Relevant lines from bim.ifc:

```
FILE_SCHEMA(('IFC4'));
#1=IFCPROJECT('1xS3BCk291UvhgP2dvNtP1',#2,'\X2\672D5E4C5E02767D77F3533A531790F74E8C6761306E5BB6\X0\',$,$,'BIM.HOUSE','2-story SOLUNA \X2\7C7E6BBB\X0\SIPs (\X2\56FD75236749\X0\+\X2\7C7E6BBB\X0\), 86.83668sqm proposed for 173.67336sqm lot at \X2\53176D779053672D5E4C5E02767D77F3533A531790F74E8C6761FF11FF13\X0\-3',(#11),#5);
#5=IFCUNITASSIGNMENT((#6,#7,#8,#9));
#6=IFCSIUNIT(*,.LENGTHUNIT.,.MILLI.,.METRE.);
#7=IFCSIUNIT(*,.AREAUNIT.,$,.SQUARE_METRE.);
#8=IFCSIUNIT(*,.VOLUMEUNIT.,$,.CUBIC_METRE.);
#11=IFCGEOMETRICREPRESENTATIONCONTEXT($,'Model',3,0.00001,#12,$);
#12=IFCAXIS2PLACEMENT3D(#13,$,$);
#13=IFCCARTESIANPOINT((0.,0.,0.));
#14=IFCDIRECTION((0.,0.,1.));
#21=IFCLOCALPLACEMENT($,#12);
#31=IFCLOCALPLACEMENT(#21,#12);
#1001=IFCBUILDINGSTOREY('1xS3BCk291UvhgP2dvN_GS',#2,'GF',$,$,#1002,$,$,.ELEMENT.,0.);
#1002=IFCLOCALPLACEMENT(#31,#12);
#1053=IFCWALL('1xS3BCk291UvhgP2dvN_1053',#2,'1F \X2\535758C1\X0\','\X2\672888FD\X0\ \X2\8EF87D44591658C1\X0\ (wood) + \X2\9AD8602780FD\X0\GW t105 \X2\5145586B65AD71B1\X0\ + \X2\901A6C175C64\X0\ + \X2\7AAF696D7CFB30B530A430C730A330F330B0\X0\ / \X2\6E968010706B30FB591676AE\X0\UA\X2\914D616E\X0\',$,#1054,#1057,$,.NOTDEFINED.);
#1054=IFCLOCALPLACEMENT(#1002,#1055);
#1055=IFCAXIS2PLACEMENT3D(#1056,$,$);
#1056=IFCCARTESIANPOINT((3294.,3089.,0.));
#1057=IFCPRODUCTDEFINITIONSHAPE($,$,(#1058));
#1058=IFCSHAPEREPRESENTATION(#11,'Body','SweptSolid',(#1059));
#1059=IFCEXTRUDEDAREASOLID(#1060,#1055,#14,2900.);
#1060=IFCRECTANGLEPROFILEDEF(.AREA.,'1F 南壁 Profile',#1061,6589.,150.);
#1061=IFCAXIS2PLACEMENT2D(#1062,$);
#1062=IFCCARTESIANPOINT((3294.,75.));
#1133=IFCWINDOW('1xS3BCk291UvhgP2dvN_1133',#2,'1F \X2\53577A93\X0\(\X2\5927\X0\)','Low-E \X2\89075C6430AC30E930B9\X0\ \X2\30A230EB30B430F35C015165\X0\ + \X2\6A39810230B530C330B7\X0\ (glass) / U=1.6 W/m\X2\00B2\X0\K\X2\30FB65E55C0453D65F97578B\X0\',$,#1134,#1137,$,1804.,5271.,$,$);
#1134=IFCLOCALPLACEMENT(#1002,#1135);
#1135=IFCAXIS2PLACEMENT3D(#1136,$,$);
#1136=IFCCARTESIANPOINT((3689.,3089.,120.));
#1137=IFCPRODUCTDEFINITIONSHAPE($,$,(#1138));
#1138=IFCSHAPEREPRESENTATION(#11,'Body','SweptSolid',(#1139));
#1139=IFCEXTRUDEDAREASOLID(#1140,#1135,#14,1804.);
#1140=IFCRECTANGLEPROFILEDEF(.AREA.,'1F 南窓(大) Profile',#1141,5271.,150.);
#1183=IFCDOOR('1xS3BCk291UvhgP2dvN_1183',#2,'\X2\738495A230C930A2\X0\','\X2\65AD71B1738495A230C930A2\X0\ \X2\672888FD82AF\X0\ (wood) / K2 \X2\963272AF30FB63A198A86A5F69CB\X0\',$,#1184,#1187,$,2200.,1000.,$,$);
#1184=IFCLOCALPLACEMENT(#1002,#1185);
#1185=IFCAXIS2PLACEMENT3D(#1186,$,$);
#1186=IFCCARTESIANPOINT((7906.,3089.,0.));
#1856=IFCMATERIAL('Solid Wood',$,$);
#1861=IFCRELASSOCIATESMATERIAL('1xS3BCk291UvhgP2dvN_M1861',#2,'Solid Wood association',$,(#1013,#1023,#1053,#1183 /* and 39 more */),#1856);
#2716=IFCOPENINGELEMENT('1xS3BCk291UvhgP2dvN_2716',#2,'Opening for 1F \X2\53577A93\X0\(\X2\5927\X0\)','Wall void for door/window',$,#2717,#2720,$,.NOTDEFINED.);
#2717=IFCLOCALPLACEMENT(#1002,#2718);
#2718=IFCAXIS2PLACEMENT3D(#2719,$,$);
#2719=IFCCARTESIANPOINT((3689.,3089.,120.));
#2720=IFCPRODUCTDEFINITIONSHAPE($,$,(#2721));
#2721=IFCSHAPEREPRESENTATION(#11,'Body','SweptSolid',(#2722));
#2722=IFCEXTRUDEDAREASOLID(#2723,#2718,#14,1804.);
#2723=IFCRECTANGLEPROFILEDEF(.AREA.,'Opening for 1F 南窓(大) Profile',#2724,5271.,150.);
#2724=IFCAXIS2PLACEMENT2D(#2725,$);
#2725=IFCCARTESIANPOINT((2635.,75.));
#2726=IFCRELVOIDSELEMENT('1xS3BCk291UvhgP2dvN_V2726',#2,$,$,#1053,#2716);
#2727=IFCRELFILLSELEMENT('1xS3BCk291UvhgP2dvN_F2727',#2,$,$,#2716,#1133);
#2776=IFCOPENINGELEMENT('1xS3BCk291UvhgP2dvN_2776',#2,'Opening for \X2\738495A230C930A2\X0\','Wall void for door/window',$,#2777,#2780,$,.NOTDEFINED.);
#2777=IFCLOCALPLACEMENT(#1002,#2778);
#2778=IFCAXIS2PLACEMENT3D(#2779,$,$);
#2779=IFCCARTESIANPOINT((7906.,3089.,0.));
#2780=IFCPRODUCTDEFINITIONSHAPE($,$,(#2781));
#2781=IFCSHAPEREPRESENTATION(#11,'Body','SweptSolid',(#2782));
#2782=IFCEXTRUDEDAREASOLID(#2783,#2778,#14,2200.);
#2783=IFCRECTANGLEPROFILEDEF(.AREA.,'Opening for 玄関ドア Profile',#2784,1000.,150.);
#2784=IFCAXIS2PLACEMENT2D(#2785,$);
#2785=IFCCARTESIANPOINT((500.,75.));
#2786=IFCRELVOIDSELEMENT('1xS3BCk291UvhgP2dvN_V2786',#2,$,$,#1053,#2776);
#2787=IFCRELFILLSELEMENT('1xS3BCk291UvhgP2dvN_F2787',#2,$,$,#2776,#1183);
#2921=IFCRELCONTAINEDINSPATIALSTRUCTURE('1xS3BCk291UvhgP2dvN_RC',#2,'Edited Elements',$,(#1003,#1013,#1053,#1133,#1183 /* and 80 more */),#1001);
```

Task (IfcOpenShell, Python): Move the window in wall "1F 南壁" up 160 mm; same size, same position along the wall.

```python
import numpy as np
import ifcopenshell
import ifcopenshell.api.geometry
import ifcopenshell.util.placement
import ifcopenshell.util.unit

model = ifcopenshell.open("bim.ifc")
unit_scale = ifcopenshell.util.unit.calculate_unit_scale(model)

window = model.by_id(1133)
opening = window.FillsVoids[0].RelatingOpeningElement
dz = 0.16 / unit_scale

shift = np.array([0.0, 0.0, dz])
# The window is not placed relative to its opening, so move both.
for product in (opening, window):
    matrix = ifcopenshell.util.placement.get_local_placement(product.ObjectPlacement)
    matrix[:3, 3] += shift
    ifcopenshell.api.geometry.edit_object_placement(model, product=product, matrix=matrix, is_si=False)

print(f"moved by {dz * unit_scale:+.3f} m")

model.write("bim_edited.ifc")
```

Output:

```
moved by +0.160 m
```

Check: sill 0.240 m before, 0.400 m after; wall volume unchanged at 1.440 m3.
